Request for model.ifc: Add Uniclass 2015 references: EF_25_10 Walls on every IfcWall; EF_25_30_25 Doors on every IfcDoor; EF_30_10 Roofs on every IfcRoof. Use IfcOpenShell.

First a look at what the model holds.

```python
import ifcopenshell

model = ifcopenshell.open("model.ifc")
print(model.schema)
print("classifications:", [c.Name for c in model.by_type("IfcClassification")])
for ifc_class in ("IfcDoor", "IfcRoof", "IfcStair", "IfcWall", "IfcWindow"):
    print(ifc_class, len(model.by_type(ifc_class)))
```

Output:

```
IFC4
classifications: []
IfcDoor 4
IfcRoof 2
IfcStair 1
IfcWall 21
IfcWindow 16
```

```python
import ifcopenshell
import ifcopenshell.api.classification

model = ifcopenshell.open("model.ifc")

system = ifcopenshell.api.classification.add_classification(model, classification="Uniclass 2015")

codes = {
    "IfcWall": ("EF_25_10", "Walls"),
    "IfcDoor": ("EF_25_30_25", "Doors"),
    "IfcRoof": ("EF_30_10", "Roofs"),
}
for ifc_class, (code, name) in codes.items():
    products = model.by_type(ifc_class)
    ifcopenshell.api.classification.add_reference(
        model, products=products, classification=system, identification=code, name=name
    )
    print(code, len(products))

model.write("model_rev.ifc")
```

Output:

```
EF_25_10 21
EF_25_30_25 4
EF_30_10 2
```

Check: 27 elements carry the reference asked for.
